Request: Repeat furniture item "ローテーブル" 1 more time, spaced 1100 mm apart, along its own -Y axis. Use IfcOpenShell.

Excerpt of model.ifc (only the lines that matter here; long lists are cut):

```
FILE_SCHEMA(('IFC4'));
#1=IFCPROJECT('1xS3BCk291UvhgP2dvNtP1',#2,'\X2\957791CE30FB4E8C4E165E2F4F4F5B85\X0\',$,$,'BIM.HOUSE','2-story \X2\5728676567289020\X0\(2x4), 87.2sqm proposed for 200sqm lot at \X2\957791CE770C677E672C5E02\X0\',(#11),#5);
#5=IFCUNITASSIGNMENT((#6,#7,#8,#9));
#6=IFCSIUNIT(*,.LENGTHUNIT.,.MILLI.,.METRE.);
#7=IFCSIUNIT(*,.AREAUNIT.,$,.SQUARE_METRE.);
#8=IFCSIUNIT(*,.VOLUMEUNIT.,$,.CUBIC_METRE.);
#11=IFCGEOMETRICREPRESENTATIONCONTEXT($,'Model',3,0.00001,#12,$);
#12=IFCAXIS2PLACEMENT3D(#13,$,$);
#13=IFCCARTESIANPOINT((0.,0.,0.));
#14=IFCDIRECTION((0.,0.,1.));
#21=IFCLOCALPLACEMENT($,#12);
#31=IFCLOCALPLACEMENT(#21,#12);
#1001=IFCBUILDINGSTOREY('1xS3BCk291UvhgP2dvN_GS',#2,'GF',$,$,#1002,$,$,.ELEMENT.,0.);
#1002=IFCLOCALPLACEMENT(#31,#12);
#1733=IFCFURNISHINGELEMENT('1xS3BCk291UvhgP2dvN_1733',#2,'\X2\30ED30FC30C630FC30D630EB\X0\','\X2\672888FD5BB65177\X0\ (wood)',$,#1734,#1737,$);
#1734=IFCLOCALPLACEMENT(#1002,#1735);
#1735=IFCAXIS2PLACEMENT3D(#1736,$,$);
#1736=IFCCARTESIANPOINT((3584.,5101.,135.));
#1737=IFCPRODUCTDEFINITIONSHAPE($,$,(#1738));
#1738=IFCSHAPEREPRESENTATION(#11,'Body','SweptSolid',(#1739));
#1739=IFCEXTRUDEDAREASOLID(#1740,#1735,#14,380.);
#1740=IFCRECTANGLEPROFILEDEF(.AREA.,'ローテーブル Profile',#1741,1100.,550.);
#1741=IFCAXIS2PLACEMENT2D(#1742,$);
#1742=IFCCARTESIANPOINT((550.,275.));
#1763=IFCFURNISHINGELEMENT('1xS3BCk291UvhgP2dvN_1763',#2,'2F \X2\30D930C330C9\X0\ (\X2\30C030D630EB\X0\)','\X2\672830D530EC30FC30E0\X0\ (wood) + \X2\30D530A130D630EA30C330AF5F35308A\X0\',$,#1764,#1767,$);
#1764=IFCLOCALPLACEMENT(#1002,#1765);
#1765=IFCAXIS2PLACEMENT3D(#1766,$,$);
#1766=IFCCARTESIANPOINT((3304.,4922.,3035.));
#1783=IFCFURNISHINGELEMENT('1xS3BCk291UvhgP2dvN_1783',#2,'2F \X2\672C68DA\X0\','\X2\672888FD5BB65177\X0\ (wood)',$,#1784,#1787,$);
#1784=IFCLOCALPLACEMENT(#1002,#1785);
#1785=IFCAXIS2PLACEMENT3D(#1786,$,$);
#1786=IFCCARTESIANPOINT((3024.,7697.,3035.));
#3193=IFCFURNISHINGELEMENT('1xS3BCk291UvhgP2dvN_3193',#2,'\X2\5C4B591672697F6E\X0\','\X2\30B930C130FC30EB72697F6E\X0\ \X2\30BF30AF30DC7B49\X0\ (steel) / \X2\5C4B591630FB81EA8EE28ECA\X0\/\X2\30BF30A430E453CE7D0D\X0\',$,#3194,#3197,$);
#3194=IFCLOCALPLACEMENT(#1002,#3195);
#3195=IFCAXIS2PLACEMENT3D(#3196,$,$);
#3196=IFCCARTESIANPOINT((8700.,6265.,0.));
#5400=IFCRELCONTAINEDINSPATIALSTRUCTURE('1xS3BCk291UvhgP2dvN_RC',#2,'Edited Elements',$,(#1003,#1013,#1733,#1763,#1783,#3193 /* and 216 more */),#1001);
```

```python
import ifcopenshell
import ifcopenshell.api.geometry
import ifcopenshell.api.root
import ifcopenshell.util.element
import ifcopenshell.util.placement

model = ifcopenshell.open("model.ifc")


def reuse_history(source, copy):
    """copy_class also copies each property set's owner history, people and application; keep the originals."""
    for rel in copy.IsDefinedBy:
        if rel.is_a("IfcRelDefinesByProperties") and (history := rel.RelatingPropertyDefinition.OwnerHistory):
            rel.RelatingPropertyDefinition.OwnerHistory = source.OwnerHistory
            ifcopenshell.util.element.remove_deep2(model, history)


source = model.by_id(1733)
base = ifcopenshell.util.placement.get_local_placement(source.ObjectPlacement)
step = -base[:3, 1] * 1100.0

for i in range(1, 2):
    copy = ifcopenshell.api.root.copy_class(model, product=source)
    copy.Representation = ifcopenshell.util.element.copy_deep(
        model, source.Representation, exclude=["IfcGeometricRepresentationContext", "IfcRepresentationMap"]
    )
    reuse_history(source, copy)
    matrix = base.copy()
    matrix[:3, 3] += i * step
    print("added at", matrix[:3, 3].round(3) + 0.0)
    ifcopenshell.api.geometry.edit_object_placement(model, product=copy, matrix=matrix, is_si=False)

model.write("model-out.ifc")
```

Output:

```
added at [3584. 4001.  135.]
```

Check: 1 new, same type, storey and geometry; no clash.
